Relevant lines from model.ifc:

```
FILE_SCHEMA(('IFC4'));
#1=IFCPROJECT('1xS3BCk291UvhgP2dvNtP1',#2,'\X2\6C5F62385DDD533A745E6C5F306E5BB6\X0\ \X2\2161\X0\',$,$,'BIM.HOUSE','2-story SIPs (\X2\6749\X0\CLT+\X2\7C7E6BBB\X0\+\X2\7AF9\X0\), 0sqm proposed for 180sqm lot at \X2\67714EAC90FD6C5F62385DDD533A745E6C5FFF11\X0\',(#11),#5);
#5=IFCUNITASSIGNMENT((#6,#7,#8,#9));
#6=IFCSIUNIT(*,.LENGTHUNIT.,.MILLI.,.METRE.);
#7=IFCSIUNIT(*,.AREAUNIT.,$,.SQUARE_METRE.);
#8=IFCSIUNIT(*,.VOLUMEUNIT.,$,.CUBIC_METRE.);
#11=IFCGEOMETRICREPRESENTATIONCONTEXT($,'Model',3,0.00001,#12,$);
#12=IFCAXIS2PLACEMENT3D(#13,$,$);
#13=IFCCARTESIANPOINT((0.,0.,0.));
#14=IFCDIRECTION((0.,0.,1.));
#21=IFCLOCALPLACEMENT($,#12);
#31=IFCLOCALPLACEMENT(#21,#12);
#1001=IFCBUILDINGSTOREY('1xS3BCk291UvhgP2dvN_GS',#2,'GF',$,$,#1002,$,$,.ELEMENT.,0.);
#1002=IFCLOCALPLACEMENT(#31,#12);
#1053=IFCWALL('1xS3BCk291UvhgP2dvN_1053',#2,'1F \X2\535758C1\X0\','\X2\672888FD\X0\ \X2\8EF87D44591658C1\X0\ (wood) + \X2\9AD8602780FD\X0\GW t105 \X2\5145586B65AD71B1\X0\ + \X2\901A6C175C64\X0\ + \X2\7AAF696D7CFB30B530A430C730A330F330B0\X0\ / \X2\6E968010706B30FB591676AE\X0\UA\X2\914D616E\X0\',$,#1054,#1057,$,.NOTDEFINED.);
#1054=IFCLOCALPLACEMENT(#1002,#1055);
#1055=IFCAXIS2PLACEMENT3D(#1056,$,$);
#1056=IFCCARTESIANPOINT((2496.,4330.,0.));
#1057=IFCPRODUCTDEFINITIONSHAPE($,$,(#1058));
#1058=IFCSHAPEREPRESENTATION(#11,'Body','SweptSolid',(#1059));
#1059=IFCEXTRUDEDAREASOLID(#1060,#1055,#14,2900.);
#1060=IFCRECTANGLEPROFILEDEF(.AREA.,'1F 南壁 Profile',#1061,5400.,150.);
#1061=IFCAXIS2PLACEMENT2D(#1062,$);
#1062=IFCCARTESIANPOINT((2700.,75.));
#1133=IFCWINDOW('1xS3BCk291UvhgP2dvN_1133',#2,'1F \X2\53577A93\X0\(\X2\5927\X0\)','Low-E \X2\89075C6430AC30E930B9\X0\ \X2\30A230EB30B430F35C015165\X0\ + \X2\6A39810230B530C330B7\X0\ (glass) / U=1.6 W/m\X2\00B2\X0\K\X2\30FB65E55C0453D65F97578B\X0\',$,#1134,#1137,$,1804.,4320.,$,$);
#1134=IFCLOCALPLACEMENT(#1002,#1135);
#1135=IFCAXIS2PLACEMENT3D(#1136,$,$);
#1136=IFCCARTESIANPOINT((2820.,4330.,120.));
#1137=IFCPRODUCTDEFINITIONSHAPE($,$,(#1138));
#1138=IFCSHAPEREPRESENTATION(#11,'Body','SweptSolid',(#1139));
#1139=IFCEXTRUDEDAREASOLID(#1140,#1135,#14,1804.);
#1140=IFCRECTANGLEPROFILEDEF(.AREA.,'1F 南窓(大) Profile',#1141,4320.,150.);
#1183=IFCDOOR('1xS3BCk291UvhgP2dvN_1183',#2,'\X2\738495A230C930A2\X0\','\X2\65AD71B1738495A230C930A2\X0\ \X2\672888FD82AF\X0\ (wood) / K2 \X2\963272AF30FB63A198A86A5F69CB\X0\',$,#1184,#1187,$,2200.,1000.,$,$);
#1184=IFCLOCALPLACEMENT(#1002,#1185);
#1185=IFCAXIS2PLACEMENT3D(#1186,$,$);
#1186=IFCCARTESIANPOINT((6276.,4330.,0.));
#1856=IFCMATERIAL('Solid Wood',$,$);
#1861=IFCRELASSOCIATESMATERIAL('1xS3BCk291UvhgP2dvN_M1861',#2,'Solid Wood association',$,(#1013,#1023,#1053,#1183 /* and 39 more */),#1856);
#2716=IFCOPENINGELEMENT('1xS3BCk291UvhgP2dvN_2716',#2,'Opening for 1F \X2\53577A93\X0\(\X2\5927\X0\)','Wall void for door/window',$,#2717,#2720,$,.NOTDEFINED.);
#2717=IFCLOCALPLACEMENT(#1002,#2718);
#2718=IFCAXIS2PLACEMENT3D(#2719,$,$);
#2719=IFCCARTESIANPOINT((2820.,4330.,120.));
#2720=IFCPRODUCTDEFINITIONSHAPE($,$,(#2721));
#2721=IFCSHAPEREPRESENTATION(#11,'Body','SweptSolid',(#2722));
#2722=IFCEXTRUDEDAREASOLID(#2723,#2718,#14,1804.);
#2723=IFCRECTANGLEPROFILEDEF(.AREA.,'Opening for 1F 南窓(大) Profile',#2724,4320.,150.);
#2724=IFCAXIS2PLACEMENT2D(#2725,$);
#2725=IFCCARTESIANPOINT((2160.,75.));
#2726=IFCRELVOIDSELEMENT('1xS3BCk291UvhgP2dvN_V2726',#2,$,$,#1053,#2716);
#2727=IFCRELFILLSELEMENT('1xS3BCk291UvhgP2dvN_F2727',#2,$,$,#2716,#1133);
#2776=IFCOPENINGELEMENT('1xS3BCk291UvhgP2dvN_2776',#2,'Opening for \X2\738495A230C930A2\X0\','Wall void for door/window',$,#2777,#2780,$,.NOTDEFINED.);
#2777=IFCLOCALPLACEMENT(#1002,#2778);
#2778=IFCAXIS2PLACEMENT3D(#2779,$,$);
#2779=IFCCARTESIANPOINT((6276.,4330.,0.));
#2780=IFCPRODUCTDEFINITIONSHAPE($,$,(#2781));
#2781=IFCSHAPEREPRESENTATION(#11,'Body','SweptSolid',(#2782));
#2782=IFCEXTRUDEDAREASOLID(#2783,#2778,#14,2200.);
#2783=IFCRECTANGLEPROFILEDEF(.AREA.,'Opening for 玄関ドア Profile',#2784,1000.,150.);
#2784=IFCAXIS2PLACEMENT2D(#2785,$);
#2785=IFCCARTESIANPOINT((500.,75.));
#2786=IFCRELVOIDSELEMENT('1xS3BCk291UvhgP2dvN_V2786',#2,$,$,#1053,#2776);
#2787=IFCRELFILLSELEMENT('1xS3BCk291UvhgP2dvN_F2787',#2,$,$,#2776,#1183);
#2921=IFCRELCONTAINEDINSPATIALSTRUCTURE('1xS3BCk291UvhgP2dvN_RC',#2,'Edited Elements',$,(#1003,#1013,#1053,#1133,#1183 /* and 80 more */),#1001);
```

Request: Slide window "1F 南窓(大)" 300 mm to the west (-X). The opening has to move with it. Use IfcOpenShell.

```python
import ifcopenshell
import ifcopenshell.api.geometry
import ifcopenshell.util.placement
import ifcopenshell.util.unit

model = ifcopenshell.open("model.ifc")
unit_scale = ifcopenshell.util.unit.calculate_unit_scale(model)

window = model.by_id(1133)
opening = window.FillsVoids[0].RelatingOpeningElement
wall = opening.VoidsElements[0].RelatingBuildingElement

wall_matrix = ifcopenshell.util.placement.get_local_placement(wall.ObjectPlacement)
shift = wall_matrix[:3, 0] * -0.3 / unit_scale
before = ifcopenshell.util.placement.get_local_placement(window.ObjectPlacement)[:3, 3].copy()

# The window is not placed relative to its opening, so move both.
for product in (opening, window):
    matrix = ifcopenshell.util.placement.get_local_placement(product.ObjectPlacement)
    matrix[:3, 3] += shift
    ifcopenshell.api.geometry.edit_object_placement(model, product=product, matrix=matrix, is_si=False)

after = ifcopenshell.util.placement.get_local_placement(window.ObjectPlacement)[:3, 3]
print("window moved by", (after - before).round(3) + 0.0)

model.write("model_rev.ifc")
```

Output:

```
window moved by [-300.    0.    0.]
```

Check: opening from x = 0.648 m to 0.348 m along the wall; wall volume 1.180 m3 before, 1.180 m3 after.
